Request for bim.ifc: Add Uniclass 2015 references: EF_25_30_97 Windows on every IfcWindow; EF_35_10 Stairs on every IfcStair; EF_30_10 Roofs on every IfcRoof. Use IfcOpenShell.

First a look at what the model holds.

```python
import ifcopenshell

model = ifcopenshell.open("bim.ifc")
print(model.schema)
print("classifications:", [c.Name for c in model.by_type("IfcClassification")])
for ifc_class in ("IfcDoor", "IfcRoof", "IfcStair", "IfcWall", "IfcWindow"):
    print(ifc_class, len(model.by_type(ifc_class)))
```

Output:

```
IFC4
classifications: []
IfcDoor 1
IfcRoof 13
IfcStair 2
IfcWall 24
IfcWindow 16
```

```python
import ifcopenshell
import ifcopenshell.api.classification

model = ifcopenshell.open("bim.ifc")

system = ifcopenshell.api.classification.add_classification(model, classification="Uniclass 2015")

codes = {
    "IfcWindow": ("EF_25_30_97", "Windows"),
    "IfcStair": ("EF_35_10", "Stairs"),
    "IfcRoof": ("EF_30_10", "Roofs"),
}
for ifc_class, (code, name) in codes.items():
    products = model.by_type(ifc_class)
    ifcopenshell.api.classification.add_reference(
        model, products=products, classification=system, identification=code, name=name
    )
    print(code, len(products))

model.write("bim-out.ifc")
```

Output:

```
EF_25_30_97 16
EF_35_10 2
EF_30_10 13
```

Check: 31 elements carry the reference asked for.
